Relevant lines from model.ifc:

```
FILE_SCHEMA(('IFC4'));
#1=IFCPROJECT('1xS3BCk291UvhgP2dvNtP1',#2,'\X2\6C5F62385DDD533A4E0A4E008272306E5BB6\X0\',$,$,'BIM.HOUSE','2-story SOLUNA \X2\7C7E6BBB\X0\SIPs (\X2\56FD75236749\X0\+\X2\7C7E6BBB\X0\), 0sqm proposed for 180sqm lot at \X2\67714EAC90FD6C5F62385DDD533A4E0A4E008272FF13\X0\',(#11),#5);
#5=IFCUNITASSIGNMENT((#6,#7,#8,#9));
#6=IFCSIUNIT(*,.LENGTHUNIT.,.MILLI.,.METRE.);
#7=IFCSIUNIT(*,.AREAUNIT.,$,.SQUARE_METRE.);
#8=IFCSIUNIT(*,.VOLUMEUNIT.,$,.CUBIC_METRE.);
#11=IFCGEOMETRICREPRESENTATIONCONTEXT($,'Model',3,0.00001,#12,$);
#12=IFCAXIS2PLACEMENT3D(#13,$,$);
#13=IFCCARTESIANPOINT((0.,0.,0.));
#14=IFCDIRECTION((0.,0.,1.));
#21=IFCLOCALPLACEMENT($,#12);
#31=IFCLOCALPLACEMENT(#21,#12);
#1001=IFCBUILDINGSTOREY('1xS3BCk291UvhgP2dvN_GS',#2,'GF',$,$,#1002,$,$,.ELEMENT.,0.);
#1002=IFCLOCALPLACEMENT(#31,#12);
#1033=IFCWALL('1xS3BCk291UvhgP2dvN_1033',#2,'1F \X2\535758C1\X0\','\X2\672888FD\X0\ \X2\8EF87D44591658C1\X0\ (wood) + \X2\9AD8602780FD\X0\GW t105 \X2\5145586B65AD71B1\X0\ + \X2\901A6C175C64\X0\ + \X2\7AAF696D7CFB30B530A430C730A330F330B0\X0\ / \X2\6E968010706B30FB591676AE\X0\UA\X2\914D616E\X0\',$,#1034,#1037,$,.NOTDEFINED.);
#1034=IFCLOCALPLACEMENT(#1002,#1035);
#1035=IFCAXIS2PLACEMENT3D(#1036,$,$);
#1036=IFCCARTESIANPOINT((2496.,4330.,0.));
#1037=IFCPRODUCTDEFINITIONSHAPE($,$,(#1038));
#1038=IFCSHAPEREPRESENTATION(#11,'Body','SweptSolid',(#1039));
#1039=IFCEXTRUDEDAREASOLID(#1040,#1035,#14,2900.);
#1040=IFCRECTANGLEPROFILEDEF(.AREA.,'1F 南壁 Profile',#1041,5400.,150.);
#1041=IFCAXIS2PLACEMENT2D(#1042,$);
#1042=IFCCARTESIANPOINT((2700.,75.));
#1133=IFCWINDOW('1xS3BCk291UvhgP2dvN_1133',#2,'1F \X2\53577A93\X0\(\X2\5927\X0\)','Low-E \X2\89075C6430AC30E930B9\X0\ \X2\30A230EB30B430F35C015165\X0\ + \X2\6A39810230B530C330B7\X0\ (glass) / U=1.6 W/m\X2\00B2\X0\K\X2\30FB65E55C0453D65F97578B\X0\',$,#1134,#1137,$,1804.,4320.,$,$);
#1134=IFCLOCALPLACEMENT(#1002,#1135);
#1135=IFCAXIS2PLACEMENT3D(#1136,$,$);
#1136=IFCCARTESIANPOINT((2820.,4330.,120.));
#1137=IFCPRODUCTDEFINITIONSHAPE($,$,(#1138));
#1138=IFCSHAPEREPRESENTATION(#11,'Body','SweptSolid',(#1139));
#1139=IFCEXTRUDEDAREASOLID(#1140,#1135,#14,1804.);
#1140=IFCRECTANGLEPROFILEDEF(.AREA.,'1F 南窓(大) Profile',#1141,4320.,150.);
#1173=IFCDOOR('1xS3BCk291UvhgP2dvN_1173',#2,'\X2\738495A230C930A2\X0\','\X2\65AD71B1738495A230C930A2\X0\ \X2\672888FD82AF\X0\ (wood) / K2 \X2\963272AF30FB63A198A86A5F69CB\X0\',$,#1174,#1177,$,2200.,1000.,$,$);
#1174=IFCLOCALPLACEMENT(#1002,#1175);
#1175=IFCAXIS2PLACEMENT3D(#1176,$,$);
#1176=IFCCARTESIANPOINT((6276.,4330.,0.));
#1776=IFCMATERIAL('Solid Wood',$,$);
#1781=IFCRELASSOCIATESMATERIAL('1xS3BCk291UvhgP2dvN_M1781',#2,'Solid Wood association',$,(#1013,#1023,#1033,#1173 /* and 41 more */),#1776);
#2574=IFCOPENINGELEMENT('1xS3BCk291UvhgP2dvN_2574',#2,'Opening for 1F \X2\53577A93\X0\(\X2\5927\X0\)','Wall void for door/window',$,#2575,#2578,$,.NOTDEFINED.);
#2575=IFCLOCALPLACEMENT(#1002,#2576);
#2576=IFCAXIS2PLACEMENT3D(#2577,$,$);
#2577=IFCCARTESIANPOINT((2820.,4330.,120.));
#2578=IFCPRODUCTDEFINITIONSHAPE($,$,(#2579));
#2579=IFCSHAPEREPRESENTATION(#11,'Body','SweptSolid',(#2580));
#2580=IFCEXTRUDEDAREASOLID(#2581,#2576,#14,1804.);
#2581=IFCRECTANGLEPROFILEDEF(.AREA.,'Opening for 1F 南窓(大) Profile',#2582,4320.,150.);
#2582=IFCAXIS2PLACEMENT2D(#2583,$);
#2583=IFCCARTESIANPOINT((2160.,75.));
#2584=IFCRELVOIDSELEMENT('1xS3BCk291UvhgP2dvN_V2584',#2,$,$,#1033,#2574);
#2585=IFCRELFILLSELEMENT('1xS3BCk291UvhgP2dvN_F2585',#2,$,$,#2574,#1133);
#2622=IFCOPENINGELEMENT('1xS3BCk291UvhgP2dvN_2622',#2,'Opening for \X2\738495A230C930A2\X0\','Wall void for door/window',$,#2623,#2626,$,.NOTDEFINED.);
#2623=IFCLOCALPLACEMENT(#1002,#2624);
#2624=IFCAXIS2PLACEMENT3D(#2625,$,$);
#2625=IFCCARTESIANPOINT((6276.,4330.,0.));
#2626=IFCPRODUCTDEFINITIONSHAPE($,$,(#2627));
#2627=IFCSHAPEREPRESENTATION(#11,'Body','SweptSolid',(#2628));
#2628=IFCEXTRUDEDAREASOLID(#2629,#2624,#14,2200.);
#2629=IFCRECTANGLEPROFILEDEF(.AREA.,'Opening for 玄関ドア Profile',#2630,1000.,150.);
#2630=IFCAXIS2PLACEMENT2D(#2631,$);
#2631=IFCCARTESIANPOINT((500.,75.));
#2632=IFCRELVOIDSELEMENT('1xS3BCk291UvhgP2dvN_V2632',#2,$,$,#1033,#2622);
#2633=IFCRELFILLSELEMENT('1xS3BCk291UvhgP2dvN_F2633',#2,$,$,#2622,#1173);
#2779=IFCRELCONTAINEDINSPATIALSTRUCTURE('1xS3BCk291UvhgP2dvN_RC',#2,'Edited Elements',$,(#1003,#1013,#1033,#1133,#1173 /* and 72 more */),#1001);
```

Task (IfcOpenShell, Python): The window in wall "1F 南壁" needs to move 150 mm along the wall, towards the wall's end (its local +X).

```python
import ifcopenshell
import ifcopenshell.api.geometry
import ifcopenshell.util.placement
import ifcopenshell.util.unit

model = ifcopenshell.open("model.ifc")
unit_scale = ifcopenshell.util.unit.calculate_unit_scale(model)

window = model.by_guid("1xS3BCk291UvhgP2dvN_1133")
opening = window.FillsVoids[0].RelatingOpeningElement
wall = opening.VoidsElements[0].RelatingBuildingElement

wall_matrix = ifcopenshell.util.placement.get_local_placement(wall.ObjectPlacement)
shift = wall_matrix[:3, 0] * 0.15 / unit_scale
before = ifcopenshell.util.placement.get_local_placement(window.ObjectPlacement)[:3, 3].copy()

# The window is not placed relative to its opening, so move both.
for product in (opening, window):
    matrix = ifcopenshell.util.placement.get_local_placement(product.ObjectPlacement)
    matrix[:3, 3] += shift
    ifcopenshell.api.geometry.edit_object_placement(model, product=product, matrix=matrix, is_si=False)

after = ifcopenshell.util.placement.get_local_placement(window.ObjectPlacement)[:3, 3]
print("window moved by", (after - before).round(3) + 0.0)

model.write("model_edited.ifc")
```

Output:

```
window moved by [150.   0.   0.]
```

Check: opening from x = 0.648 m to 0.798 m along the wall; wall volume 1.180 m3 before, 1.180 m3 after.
